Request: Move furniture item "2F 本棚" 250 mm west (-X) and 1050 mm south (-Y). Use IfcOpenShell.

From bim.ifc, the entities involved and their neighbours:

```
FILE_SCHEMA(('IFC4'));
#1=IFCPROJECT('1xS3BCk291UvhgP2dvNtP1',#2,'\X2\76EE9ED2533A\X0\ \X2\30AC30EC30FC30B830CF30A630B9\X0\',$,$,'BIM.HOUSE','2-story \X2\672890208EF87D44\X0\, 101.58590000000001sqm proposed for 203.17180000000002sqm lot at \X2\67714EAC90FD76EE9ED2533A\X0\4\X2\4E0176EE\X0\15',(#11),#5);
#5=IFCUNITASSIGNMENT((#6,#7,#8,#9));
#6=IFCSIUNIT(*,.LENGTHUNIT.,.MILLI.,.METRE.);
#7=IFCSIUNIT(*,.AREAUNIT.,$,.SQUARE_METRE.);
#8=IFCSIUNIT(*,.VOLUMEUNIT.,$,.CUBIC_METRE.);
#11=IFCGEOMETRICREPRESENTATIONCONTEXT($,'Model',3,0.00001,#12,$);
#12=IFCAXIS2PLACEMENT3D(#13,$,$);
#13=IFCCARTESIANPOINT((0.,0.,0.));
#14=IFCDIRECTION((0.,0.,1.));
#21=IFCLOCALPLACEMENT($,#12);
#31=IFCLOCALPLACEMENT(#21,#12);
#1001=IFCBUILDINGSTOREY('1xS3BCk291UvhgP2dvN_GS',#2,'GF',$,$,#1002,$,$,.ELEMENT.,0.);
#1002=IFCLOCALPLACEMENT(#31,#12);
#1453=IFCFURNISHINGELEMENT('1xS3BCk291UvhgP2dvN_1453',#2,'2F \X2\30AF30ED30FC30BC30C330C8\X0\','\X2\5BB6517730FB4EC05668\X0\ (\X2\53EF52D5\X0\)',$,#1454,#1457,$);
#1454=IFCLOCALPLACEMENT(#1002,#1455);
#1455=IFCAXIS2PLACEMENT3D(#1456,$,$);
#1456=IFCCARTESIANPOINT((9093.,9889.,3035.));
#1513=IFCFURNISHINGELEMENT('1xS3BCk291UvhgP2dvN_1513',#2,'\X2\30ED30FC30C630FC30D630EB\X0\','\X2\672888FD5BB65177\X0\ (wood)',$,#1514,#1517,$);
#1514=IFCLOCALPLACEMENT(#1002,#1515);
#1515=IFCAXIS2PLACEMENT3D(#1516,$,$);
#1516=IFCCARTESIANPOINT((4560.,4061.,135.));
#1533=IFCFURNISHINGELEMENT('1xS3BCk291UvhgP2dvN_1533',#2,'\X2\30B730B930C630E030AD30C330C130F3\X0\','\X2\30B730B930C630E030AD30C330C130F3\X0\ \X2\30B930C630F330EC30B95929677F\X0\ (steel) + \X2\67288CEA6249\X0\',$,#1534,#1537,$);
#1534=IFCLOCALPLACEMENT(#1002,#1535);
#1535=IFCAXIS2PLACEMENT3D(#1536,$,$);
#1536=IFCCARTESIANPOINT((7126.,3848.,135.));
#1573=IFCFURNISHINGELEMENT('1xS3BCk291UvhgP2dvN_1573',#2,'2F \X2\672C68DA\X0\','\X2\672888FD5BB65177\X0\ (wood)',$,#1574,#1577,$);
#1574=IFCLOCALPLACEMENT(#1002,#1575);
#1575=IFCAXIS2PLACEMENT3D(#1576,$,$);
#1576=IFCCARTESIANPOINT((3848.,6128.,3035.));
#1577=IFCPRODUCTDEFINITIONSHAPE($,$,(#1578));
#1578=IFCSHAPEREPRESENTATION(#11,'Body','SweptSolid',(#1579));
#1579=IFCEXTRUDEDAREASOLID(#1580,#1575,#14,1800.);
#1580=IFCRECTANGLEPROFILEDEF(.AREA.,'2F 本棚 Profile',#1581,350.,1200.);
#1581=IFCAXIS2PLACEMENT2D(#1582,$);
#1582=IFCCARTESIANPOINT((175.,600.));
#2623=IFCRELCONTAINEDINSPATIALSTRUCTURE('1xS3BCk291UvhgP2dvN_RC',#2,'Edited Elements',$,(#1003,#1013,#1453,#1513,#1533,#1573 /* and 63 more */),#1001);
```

```python
import ifcopenshell
import ifcopenshell.api.geometry
import ifcopenshell.util.placement
import ifcopenshell.util.unit

model = ifcopenshell.open("bim.ifc")
unit_scale = ifcopenshell.util.unit.calculate_unit_scale(model)

item = model.by_guid("1xS3BCk291UvhgP2dvN_1573")
matrix = ifcopenshell.util.placement.get_local_placement(item.ObjectPlacement)
matrix[0, 3] -= 0.25 / unit_scale
matrix[1, 3] -= 1.05 / unit_scale
ifcopenshell.api.geometry.edit_object_placement(model, product=item, matrix=matrix, is_si=False)

print(ifcopenshell.util.placement.get_local_placement(item.ObjectPlacement).round(3) + 0.0)

model.write("bim_updated.ifc")
```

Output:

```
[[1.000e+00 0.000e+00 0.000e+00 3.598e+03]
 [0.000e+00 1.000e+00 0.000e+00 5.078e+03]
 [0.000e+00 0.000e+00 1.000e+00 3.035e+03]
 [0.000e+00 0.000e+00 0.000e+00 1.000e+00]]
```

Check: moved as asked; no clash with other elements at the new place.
